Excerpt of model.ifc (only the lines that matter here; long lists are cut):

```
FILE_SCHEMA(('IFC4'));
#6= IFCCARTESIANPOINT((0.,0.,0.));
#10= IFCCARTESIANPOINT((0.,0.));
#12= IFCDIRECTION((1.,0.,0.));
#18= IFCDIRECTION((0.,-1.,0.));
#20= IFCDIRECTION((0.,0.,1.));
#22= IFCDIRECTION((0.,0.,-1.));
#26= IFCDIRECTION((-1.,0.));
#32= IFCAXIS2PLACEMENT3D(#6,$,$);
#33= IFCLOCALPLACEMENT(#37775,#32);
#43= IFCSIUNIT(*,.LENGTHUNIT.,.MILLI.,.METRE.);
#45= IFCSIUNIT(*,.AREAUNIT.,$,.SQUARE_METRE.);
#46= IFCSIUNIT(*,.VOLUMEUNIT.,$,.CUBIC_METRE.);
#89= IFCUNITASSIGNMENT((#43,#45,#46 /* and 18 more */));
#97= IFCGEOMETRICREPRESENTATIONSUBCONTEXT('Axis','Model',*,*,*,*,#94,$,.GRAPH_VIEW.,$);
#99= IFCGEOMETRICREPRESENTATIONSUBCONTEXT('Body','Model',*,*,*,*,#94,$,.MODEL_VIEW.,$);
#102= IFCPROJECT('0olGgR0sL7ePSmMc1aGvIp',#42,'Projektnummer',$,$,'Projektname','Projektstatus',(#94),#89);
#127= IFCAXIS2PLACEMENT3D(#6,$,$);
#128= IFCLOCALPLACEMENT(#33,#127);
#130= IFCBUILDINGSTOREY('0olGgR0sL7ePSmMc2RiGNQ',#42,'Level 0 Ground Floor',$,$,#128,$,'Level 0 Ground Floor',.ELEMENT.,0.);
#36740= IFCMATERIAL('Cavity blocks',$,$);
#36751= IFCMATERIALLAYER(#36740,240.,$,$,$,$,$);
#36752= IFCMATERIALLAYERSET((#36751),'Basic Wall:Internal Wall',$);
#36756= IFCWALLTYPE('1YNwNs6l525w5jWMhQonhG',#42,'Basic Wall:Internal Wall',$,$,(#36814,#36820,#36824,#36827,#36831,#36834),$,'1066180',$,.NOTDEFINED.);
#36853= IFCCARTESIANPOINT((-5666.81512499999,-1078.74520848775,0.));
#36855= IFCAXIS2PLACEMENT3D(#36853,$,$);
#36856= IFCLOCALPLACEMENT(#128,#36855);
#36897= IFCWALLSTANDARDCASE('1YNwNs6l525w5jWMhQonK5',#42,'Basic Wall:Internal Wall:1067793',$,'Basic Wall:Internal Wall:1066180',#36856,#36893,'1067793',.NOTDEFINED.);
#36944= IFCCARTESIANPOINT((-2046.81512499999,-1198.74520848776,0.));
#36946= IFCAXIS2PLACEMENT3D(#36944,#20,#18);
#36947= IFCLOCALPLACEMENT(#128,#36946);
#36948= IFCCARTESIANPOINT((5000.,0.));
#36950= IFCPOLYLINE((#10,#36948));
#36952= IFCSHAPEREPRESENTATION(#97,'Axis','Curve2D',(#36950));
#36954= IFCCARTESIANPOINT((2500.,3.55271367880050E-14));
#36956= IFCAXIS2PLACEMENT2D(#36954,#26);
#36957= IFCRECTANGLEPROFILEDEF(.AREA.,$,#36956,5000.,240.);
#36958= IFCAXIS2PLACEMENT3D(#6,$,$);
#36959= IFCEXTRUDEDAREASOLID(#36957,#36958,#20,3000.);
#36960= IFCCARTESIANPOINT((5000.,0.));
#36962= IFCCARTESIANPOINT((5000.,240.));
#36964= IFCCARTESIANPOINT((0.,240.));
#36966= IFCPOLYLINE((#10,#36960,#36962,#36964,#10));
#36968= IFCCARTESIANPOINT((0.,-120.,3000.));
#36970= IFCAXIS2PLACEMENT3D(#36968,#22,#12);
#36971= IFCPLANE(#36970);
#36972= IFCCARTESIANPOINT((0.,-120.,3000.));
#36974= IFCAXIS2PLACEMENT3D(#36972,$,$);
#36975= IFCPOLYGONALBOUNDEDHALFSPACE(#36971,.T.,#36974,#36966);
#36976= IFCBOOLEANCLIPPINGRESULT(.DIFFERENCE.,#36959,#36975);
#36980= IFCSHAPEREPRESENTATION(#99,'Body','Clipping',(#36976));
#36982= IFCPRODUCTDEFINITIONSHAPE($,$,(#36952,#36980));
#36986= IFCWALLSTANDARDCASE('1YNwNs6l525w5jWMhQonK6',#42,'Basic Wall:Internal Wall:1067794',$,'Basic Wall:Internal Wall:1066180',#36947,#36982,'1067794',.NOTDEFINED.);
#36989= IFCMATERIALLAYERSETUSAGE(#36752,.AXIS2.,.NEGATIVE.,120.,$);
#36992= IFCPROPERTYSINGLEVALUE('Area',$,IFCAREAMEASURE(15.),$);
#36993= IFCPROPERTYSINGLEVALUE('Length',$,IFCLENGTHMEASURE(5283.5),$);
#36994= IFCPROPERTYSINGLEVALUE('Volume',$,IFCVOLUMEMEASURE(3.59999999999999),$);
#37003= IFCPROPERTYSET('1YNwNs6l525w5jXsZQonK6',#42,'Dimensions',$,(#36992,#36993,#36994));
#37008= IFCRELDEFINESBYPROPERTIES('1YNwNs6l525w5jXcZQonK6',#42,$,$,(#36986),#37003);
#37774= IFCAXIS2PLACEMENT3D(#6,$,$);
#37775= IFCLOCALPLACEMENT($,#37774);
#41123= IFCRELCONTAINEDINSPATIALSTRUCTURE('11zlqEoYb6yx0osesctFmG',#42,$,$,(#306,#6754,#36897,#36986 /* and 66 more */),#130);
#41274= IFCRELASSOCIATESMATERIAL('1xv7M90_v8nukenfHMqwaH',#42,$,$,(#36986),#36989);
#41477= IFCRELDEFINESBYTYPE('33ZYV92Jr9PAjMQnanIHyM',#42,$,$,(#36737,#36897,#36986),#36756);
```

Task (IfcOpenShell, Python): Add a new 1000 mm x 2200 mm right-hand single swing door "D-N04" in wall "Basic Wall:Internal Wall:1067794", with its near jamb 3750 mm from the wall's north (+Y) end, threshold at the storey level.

```python
import numpy as np
import ifcopenshell
import ifcopenshell.api.feature
import ifcopenshell.api.geometry
import ifcopenshell.api.pset
import ifcopenshell.api.root
import ifcopenshell.api.spatial
import ifcopenshell.geom
import ifcopenshell.util.element
import ifcopenshell.util.placement
import ifcopenshell.util.representation
import ifcopenshell.util.shape
import ifcopenshell.util.unit

model = ifcopenshell.open("model.ifc")
unit_scale = ifcopenshell.util.unit.calculate_unit_scale(model)
area_scale = ifcopenshell.util.unit.calculate_unit_scale(model, "AREAUNIT")
volume_scale = ifcopenshell.util.unit.calculate_unit_scale(model, "VOLUMEUNIT")
settings = ifcopenshell.geom.settings()


def volume(element):
    """Net volume in cubic metres, openings subtracted."""
    shape = ifcopenshell.geom.create_shape(settings, element)
    return ifcopenshell.util.shape.get_volume(shape.geometry)


wall = model.by_guid("1YNwNs6l525w5jWMhQonK6")
storey = ifcopenshell.util.element.get_container(wall, ifc_class="IfcBuildingStorey")
context = ifcopenshell.util.representation.get_context(model, "Model", "Body", "MODEL_VIEW")
before = volume(wall)

width, height, from_end, sill = 1, 2.2, 3.75, 0.0  # metres

# The wall runs along its own X axis, and the end named is its -X end.
wall_shape = ifcopenshell.geom.create_shape(settings, wall)
x, y, z = ifcopenshell.util.shape.get_vertices(wall_shape.geometry).T
start = x.min() + from_end
face, thickness = float(y.min()), float(y.max() - y.min())
wall_matrix = ifcopenshell.util.placement.get_local_placement(wall.ObjectPlacement)
level = ifcopenshell.util.placement.get_local_placement(storey.ObjectPlacement)[2, 3]


def in_wall(x, y):
    """Placement at x, y metres in the wall's axes, at sill height."""
    matrix = wall_matrix.copy()
    matrix[:, 3] = wall_matrix @ np.array([x / unit_scale, y / unit_scale, 0.0, 1.0])
    matrix[2, 3] = level + sill / unit_scale
    return matrix


# Opening: a box that overshoots both wall faces by 50 mm.
opening = ifcopenshell.api.root.create_entity(model, ifc_class="IfcOpeningElement", predefined_type="OPENING")
box = ifcopenshell.api.geometry.add_wall_representation(
    model, context=context, length=width, height=height, thickness=thickness + 0.1
)
ifcopenshell.api.geometry.assign_representation(model, product=opening, representation=box)
ifcopenshell.api.geometry.edit_object_placement(model, product=opening, matrix=in_wall(start, face - 0.05), is_si=False)
ifcopenshell.api.feature.add_feature(model, feature=opening, element=wall)

door = ifcopenshell.api.root.create_entity(model, ifc_class="IfcDoor", name="D-N04", predefined_type="DOOR")
door.OverallWidth, door.OverallHeight = width / unit_scale, height / unit_scale
door.OperationType = "SINGLE_SWING_RIGHT"
body = ifcopenshell.api.geometry.add_door_representation(
    model,
    context=context,
    overall_width=door.OverallWidth,
    overall_height=door.OverallHeight,
    operation_type="SINGLE_SWING_RIGHT",
    lining_properties={"LiningDepth": thickness / unit_scale, "ThresholdDepth": thickness / unit_scale},
)
ifcopenshell.api.geometry.assign_representation(model, product=door, representation=body)
ifcopenshell.api.spatial.assign_container(model, products=[door], relating_structure=storey)
ifcopenshell.api.feature.add_filling(model, opening=opening, element=door)

# The lining spans the wall, so the door starts at the wall face.
ifcopenshell.api.geometry.edit_object_placement(model, product=door, matrix=in_wall(start, face), is_si=False)

after = volume(wall)

# Update the wall's stored quantities.
pset = model.by_id(ifcopenshell.util.element.get_pset(wall, "Dimensions", should_inherit=False)["id"])
ifcopenshell.api.pset.edit_pset(model, pset=pset, properties={
    "Area": model.create_entity("IfcAreaMeasure", after / thickness / area_scale),
    "Volume": model.create_entity("IfcVolumeMeasure", after / volume_scale),
})

print(f"wall volume {before:.3f} -> {after:.3f} m3")

model.write("model-out.ifc")
```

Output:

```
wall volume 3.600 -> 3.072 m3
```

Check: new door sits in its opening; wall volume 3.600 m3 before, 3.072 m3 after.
